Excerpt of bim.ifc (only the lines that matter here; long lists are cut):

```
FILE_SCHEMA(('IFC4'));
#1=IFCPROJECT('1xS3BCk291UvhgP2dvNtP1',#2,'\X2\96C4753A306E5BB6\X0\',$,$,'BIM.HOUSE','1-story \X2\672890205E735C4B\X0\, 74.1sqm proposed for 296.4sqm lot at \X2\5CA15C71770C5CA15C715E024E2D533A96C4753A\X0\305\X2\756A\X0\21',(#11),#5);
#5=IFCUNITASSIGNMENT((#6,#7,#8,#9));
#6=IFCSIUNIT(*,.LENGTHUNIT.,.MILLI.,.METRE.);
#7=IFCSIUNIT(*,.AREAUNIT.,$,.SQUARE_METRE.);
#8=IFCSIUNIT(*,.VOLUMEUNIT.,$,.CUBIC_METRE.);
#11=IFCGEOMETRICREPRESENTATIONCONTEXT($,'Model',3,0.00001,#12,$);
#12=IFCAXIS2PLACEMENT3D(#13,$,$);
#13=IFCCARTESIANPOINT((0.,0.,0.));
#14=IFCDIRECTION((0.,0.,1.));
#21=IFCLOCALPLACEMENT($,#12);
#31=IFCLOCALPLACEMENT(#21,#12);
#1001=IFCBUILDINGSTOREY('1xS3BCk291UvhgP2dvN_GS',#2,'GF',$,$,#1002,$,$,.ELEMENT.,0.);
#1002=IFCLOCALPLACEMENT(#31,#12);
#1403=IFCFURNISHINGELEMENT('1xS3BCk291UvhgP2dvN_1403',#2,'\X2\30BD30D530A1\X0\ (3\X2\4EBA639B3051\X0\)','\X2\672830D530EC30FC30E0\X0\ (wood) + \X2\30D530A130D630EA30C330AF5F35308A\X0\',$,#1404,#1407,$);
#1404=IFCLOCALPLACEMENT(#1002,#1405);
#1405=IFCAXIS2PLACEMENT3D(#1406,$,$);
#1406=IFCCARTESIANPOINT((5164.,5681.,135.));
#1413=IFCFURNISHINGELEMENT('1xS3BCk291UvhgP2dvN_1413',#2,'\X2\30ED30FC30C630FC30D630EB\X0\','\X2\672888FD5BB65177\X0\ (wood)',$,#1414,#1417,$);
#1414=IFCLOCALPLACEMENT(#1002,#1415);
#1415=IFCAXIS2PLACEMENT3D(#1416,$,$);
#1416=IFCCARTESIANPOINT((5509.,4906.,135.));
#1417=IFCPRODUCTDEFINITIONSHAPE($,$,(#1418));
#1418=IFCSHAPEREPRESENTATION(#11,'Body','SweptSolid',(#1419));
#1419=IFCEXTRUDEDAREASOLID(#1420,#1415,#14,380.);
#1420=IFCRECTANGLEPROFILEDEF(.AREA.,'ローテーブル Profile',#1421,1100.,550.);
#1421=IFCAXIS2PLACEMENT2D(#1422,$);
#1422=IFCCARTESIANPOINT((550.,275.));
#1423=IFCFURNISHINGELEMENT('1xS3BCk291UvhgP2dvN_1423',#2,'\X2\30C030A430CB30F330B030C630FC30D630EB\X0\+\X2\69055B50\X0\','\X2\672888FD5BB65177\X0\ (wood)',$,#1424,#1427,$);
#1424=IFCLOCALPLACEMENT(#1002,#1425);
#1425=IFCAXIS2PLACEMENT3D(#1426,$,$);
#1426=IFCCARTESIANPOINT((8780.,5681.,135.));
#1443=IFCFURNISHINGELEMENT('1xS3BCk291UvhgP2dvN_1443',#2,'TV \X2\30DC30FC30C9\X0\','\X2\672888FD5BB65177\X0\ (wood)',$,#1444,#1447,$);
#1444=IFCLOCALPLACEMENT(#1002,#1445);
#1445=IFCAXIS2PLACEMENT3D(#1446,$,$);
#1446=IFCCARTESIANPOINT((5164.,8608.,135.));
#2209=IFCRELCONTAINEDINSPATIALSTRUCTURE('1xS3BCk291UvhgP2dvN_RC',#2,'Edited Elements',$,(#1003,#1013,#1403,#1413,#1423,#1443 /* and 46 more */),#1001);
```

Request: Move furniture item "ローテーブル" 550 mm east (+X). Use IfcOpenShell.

```python
import ifcopenshell
import ifcopenshell.api.geometry
import ifcopenshell.util.placement
import ifcopenshell.util.unit

model = ifcopenshell.open("bim.ifc")
unit_scale = ifcopenshell.util.unit.calculate_unit_scale(model)

item = model.by_id(1413)
matrix = ifcopenshell.util.placement.get_local_placement(item.ObjectPlacement)
matrix[0, 3] += 0.55 / unit_scale
ifcopenshell.api.geometry.edit_object_placement(model, product=item, matrix=matrix, is_si=False)

print(ifcopenshell.util.placement.get_local_placement(item.ObjectPlacement).round(3) + 0.0)

model.write("bim-out.ifc")
```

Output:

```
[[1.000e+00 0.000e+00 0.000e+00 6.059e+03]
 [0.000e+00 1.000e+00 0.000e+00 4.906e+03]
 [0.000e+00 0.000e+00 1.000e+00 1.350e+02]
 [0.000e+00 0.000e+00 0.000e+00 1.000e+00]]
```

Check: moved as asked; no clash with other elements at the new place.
